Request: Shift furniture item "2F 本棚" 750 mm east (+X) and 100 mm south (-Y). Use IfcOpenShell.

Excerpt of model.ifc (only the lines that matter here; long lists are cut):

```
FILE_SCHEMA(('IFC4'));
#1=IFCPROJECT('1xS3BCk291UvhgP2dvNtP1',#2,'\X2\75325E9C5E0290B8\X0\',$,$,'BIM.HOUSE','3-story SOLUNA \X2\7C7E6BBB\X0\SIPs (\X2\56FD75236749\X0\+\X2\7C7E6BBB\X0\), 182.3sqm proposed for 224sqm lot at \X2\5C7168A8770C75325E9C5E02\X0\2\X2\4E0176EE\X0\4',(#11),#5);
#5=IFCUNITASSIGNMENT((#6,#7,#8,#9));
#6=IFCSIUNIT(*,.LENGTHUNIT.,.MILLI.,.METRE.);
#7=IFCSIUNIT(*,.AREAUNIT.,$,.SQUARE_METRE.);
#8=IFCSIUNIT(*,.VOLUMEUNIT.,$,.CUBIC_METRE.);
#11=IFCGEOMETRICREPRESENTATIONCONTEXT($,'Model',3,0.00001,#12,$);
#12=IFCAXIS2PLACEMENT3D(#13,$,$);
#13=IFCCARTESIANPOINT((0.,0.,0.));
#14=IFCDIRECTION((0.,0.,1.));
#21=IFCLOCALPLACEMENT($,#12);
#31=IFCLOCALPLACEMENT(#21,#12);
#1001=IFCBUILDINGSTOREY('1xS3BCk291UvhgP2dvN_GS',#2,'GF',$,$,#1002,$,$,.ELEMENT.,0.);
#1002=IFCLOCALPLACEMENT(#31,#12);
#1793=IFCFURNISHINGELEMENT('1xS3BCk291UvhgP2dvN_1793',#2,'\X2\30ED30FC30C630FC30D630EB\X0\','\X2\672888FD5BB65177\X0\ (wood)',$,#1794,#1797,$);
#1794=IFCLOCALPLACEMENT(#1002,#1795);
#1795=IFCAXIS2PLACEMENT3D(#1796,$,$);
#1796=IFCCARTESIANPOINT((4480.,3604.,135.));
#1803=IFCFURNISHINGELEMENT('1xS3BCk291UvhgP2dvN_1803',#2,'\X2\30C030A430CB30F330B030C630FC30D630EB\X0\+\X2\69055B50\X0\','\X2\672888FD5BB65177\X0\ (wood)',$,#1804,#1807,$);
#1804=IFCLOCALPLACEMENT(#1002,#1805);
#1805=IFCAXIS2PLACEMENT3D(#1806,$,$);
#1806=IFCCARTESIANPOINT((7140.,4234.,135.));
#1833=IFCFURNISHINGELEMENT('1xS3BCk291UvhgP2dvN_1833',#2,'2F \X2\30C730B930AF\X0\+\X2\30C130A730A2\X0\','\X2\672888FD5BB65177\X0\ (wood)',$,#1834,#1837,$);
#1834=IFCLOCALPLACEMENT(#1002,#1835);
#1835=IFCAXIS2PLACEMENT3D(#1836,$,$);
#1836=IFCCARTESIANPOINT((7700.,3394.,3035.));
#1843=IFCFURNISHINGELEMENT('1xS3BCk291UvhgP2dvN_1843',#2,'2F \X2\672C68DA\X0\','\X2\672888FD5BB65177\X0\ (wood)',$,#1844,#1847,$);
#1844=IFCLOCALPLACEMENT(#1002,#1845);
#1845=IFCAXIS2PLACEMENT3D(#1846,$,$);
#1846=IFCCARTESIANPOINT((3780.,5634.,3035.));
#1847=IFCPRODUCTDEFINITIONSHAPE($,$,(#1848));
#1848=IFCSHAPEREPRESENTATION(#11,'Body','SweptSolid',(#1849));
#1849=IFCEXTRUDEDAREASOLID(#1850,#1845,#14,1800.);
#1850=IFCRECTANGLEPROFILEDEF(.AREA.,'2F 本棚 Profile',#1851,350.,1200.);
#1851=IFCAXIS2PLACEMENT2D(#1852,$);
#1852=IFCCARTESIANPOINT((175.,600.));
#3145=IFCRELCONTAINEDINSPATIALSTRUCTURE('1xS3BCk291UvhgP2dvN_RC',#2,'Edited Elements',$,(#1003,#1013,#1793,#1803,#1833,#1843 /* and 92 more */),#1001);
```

```python
import ifcopenshell
import ifcopenshell.api.geometry
import ifcopenshell.util.placement
import ifcopenshell.util.unit

model = ifcopenshell.open("model.ifc")
unit_scale = ifcopenshell.util.unit.calculate_unit_scale(model)

item = model.by_id(1843)
matrix = ifcopenshell.util.placement.get_local_placement(item.ObjectPlacement)
matrix[0, 3] += 0.75 / unit_scale
matrix[1, 3] -= 0.1 / unit_scale
ifcopenshell.api.geometry.edit_object_placement(model, product=item, matrix=matrix, is_si=False)

print(ifcopenshell.util.placement.get_local_placement(item.ObjectPlacement).round(3) + 0.0)

model.write("model_v2.ifc")
```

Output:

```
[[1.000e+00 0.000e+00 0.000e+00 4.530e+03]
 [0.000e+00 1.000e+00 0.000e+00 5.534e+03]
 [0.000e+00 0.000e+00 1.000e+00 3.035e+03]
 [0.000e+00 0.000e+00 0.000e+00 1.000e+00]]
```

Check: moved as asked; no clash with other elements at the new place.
